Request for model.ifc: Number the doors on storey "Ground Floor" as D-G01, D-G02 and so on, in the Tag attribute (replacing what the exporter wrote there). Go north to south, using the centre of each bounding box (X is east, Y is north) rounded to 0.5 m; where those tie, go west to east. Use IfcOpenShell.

First a look at what the model holds.

```python
import ifcopenshell
import ifcopenshell.util.element
import ifcopenshell.util.placement

model = ifcopenshell.open("model.ifc")
print(model.schema)
storey = next(s for s in model.by_type("IfcBuildingStorey") if s.Name == "Ground Floor")
doors = [e for e in ifcopenshell.util.element.get_decomposition(storey) if e.is_a("IfcDoor")]
for e in sorted(doors, key=lambda e: e.id()):
    origin = ifcopenshell.util.placement.get_local_placement(e.ObjectPlacement)[:3, 3]
    print(e.id(), e.Tag, e.Name, origin.round(2) + 0.0, sep=" | ")
```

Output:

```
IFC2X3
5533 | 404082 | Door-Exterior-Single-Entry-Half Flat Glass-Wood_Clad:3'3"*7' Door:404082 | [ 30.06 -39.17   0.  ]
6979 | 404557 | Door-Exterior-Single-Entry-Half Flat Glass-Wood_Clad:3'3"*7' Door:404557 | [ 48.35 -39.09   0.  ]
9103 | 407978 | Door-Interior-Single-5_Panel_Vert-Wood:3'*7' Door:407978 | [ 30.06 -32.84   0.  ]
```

```python
import ifcopenshell
import ifcopenshell.geom
import ifcopenshell.util.element
import ifcopenshell.util.shape

model = ifcopenshell.open("model.ifc")
settings = ifcopenshell.geom.settings()
settings.set("use-world-coords", True)


def centre(element):
    shape = ifcopenshell.geom.create_shape(settings, element)
    return ifcopenshell.util.shape.get_bbox_centroid(shape.geometry)


storey = next(s for s in model.by_type("IfcBuildingStorey") if s.Name == "Ground Floor")
doors = [e for e in ifcopenshell.util.element.get_decomposition(storey) if e.is_a("IfcDoor")]

# Insertion points can sit at a corner or the storey origin, so sort by the geometry (in metres).
centres = {e: centre(e) for e in doors}
doors.sort(key=lambda e: (-round(centres[e][1] / 0.5), centres[e][0]))

for i, e in enumerate(doors, start=1):
    number = f"D-G{i:02d}"
    e.Tag = number
    print(e.id(), number)

model.write("model_rev.ifc")
```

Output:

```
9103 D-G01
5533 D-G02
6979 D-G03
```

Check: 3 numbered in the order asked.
